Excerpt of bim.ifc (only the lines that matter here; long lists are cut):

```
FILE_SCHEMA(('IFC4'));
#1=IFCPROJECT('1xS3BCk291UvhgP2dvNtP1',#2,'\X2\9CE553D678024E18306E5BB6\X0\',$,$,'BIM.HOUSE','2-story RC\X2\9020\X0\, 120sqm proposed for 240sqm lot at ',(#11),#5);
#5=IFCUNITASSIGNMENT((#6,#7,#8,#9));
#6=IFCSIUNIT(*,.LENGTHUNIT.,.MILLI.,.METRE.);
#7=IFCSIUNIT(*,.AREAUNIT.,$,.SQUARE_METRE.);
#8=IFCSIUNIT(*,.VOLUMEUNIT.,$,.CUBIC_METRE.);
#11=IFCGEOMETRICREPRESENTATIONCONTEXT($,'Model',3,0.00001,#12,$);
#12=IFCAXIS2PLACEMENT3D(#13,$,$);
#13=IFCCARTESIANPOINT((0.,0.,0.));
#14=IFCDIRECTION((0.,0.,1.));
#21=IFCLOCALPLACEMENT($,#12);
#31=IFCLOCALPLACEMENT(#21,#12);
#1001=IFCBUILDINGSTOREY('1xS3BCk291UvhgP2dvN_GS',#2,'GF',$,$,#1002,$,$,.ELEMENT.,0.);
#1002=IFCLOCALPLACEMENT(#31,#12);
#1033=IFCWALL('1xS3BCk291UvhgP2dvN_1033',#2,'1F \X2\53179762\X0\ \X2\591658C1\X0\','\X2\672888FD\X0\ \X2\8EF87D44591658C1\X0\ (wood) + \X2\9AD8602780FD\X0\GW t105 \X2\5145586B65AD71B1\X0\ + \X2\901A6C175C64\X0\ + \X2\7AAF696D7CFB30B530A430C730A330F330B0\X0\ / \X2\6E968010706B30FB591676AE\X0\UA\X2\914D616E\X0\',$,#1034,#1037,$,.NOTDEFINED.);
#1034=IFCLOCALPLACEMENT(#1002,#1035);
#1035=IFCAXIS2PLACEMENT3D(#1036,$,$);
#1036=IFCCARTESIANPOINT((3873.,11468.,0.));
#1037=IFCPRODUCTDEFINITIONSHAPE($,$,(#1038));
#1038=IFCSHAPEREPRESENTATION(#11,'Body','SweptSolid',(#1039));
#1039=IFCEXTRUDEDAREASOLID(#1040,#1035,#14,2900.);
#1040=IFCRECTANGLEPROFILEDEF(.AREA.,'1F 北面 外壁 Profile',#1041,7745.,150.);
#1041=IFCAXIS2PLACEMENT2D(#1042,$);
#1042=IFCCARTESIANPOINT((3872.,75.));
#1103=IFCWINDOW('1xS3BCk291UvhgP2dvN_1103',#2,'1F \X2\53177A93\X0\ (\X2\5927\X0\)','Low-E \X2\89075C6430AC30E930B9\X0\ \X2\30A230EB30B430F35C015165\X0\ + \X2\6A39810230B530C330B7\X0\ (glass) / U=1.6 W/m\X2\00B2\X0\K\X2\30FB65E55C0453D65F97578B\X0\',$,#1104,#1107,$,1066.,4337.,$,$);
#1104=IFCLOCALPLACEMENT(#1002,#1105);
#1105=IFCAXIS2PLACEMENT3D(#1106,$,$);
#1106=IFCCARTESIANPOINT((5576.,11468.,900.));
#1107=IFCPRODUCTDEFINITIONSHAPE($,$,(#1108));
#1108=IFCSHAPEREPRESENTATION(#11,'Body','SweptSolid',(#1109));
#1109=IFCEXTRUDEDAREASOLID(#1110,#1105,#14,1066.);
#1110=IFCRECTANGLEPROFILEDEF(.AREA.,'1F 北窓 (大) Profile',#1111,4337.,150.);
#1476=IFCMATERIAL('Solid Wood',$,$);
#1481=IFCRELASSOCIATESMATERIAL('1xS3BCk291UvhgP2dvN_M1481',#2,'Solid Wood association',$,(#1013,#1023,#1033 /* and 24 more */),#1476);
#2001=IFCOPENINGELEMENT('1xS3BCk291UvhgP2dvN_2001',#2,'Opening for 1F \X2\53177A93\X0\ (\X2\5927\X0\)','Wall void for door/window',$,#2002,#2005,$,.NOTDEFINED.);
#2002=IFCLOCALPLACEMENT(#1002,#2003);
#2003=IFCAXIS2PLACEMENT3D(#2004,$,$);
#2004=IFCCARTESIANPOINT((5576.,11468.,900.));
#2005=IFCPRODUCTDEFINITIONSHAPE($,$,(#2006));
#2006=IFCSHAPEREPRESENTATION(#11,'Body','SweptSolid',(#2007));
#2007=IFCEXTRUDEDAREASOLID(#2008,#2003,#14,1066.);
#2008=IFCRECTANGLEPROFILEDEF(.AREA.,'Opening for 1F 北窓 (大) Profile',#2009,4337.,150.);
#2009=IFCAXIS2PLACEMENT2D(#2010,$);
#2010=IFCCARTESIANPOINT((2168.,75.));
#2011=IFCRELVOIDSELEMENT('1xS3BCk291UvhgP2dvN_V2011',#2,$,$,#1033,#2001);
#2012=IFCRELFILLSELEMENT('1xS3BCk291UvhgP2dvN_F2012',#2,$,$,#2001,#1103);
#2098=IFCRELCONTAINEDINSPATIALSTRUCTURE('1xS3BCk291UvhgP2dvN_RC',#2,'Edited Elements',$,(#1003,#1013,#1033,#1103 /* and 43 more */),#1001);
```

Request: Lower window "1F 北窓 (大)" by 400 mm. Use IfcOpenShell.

```python
import numpy as np
import ifcopenshell
import ifcopenshell.api.geometry
import ifcopenshell.util.placement
import ifcopenshell.util.unit

model = ifcopenshell.open("bim.ifc")
unit_scale = ifcopenshell.util.unit.calculate_unit_scale(model)

window = model.by_id(1103)
opening = window.FillsVoids[0].RelatingOpeningElement
dz = -0.4 / unit_scale

shift = np.array([0.0, 0.0, dz])
# The window is not placed relative to its opening, so move both.
for product in (opening, window):
    matrix = ifcopenshell.util.placement.get_local_placement(product.ObjectPlacement)
    matrix[:3, 3] += shift
    ifcopenshell.api.geometry.edit_object_placement(model, product=product, matrix=matrix, is_si=False)

print(f"moved by {dz * unit_scale:+.3f} m")

model.write("bim_rev.ifc")
```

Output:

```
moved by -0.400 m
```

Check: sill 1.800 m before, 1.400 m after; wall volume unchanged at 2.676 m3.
